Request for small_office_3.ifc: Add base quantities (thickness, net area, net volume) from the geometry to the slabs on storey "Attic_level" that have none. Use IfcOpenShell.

First a look at what the model holds.

```python
import ifcopenshell
import ifcopenshell.util.element
import ifcopenshell.util.unit

model = ifcopenshell.open("small_office_3.ifc")
print(model.schema)
for unit_type in ("LENGTHUNIT", "AREAUNIT", "VOLUMEUNIT"):
    print(unit_type, ifcopenshell.util.unit.calculate_unit_scale(model, unit_type))
storey = next(s for s in model.by_type("IfcBuildingStorey") if s.Name == "Attic_level")
slabs = [e for e in ifcopenshell.util.element.get_decomposition(storey) if e.is_a("IfcSlab")]
for e in sorted(slabs, key=lambda e: e.id()):
    print(e.id(), e.is_a(), e.Name, list(ifcopenshell.util.element.get_psets(e, qtos_only=True)), sep=" | ")
```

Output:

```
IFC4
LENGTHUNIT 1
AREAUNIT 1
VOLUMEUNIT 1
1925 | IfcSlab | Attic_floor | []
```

```python
import ifcopenshell
import ifcopenshell.api.pset
import ifcopenshell.geom
import ifcopenshell.util.element
import ifcopenshell.util.shape
import ifcopenshell.util.unit

model = ifcopenshell.open("small_office_3.ifc")
unit_scale = ifcopenshell.util.unit.calculate_unit_scale(model)
area_scale = ifcopenshell.util.unit.calculate_unit_scale(model, "AREAUNIT")
volume_scale = ifcopenshell.util.unit.calculate_unit_scale(model, "VOLUMEUNIT")
settings = ifcopenshell.geom.settings()

storey = next(s for s in model.by_type("IfcBuildingStorey") if s.Name == "Attic_level")
slabs = [e for e in ifcopenshell.util.element.get_decomposition(storey) if e.is_a("IfcSlab")]

for e in sorted(slabs, key=lambda e: e.id()):
    if ifcopenshell.util.element.get_psets(e, qtos_only=True, should_inherit=False):
        continue
    # Geometry comes back in metres, in the element's own axes.
    shape = ifcopenshell.geom.create_shape(settings, e)
    values = {
        "Width": ifcopenshell.util.shape.get_z(shape.geometry) / unit_scale,
        "NetArea": ifcopenshell.util.shape.get_footprint_area(shape.geometry) / area_scale,
        "NetVolume": ifcopenshell.util.shape.get_volume(shape.geometry) / volume_scale,
    }
    qto = ifcopenshell.api.pset.add_qto(model, product=e, name="Qto_SlabBaseQuantities")
    ifcopenshell.api.pset.edit_qto(model, qto=qto, properties=values)
    print(e.id(), {k: round(v, 3) for k, v in values.items()})

model.write("small_office_3_edited.ifc")
```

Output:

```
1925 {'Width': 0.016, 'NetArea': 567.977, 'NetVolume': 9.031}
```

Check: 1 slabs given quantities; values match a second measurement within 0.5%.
